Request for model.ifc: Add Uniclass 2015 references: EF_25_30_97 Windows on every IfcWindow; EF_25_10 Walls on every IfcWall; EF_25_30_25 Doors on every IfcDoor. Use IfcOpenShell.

First a look at what the model holds.

```python
import ifcopenshell

model = ifcopenshell.open("model.ifc")
print(model.schema)
print("classifications:", [c.Name for c in model.by_type("IfcClassification")])
for ifc_class in ("IfcDoor", "IfcRoof", "IfcStair", "IfcWall", "IfcWindow"):
    print(ifc_class, len(model.by_type(ifc_class)))
```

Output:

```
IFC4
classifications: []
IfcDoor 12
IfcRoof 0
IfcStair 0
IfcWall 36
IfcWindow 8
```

```python
import ifcopenshell
import ifcopenshell.api.classification

model = ifcopenshell.open("model.ifc")

system = ifcopenshell.api.classification.add_classification(model, classification="Uniclass 2015")

codes = {
    "IfcWindow": ("EF_25_30_97", "Windows"),
    "IfcWall": ("EF_25_10", "Walls"),
    "IfcDoor": ("EF_25_30_25", "Doors"),
}
for ifc_class, (code, name) in codes.items():
    products = model.by_type(ifc_class)
    ifcopenshell.api.classification.add_reference(
        model, products=products, classification=system, identification=code, name=name
    )
    print(code, len(products))

model.write("model_rev.ifc")
```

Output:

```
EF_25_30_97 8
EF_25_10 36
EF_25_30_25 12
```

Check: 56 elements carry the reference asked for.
